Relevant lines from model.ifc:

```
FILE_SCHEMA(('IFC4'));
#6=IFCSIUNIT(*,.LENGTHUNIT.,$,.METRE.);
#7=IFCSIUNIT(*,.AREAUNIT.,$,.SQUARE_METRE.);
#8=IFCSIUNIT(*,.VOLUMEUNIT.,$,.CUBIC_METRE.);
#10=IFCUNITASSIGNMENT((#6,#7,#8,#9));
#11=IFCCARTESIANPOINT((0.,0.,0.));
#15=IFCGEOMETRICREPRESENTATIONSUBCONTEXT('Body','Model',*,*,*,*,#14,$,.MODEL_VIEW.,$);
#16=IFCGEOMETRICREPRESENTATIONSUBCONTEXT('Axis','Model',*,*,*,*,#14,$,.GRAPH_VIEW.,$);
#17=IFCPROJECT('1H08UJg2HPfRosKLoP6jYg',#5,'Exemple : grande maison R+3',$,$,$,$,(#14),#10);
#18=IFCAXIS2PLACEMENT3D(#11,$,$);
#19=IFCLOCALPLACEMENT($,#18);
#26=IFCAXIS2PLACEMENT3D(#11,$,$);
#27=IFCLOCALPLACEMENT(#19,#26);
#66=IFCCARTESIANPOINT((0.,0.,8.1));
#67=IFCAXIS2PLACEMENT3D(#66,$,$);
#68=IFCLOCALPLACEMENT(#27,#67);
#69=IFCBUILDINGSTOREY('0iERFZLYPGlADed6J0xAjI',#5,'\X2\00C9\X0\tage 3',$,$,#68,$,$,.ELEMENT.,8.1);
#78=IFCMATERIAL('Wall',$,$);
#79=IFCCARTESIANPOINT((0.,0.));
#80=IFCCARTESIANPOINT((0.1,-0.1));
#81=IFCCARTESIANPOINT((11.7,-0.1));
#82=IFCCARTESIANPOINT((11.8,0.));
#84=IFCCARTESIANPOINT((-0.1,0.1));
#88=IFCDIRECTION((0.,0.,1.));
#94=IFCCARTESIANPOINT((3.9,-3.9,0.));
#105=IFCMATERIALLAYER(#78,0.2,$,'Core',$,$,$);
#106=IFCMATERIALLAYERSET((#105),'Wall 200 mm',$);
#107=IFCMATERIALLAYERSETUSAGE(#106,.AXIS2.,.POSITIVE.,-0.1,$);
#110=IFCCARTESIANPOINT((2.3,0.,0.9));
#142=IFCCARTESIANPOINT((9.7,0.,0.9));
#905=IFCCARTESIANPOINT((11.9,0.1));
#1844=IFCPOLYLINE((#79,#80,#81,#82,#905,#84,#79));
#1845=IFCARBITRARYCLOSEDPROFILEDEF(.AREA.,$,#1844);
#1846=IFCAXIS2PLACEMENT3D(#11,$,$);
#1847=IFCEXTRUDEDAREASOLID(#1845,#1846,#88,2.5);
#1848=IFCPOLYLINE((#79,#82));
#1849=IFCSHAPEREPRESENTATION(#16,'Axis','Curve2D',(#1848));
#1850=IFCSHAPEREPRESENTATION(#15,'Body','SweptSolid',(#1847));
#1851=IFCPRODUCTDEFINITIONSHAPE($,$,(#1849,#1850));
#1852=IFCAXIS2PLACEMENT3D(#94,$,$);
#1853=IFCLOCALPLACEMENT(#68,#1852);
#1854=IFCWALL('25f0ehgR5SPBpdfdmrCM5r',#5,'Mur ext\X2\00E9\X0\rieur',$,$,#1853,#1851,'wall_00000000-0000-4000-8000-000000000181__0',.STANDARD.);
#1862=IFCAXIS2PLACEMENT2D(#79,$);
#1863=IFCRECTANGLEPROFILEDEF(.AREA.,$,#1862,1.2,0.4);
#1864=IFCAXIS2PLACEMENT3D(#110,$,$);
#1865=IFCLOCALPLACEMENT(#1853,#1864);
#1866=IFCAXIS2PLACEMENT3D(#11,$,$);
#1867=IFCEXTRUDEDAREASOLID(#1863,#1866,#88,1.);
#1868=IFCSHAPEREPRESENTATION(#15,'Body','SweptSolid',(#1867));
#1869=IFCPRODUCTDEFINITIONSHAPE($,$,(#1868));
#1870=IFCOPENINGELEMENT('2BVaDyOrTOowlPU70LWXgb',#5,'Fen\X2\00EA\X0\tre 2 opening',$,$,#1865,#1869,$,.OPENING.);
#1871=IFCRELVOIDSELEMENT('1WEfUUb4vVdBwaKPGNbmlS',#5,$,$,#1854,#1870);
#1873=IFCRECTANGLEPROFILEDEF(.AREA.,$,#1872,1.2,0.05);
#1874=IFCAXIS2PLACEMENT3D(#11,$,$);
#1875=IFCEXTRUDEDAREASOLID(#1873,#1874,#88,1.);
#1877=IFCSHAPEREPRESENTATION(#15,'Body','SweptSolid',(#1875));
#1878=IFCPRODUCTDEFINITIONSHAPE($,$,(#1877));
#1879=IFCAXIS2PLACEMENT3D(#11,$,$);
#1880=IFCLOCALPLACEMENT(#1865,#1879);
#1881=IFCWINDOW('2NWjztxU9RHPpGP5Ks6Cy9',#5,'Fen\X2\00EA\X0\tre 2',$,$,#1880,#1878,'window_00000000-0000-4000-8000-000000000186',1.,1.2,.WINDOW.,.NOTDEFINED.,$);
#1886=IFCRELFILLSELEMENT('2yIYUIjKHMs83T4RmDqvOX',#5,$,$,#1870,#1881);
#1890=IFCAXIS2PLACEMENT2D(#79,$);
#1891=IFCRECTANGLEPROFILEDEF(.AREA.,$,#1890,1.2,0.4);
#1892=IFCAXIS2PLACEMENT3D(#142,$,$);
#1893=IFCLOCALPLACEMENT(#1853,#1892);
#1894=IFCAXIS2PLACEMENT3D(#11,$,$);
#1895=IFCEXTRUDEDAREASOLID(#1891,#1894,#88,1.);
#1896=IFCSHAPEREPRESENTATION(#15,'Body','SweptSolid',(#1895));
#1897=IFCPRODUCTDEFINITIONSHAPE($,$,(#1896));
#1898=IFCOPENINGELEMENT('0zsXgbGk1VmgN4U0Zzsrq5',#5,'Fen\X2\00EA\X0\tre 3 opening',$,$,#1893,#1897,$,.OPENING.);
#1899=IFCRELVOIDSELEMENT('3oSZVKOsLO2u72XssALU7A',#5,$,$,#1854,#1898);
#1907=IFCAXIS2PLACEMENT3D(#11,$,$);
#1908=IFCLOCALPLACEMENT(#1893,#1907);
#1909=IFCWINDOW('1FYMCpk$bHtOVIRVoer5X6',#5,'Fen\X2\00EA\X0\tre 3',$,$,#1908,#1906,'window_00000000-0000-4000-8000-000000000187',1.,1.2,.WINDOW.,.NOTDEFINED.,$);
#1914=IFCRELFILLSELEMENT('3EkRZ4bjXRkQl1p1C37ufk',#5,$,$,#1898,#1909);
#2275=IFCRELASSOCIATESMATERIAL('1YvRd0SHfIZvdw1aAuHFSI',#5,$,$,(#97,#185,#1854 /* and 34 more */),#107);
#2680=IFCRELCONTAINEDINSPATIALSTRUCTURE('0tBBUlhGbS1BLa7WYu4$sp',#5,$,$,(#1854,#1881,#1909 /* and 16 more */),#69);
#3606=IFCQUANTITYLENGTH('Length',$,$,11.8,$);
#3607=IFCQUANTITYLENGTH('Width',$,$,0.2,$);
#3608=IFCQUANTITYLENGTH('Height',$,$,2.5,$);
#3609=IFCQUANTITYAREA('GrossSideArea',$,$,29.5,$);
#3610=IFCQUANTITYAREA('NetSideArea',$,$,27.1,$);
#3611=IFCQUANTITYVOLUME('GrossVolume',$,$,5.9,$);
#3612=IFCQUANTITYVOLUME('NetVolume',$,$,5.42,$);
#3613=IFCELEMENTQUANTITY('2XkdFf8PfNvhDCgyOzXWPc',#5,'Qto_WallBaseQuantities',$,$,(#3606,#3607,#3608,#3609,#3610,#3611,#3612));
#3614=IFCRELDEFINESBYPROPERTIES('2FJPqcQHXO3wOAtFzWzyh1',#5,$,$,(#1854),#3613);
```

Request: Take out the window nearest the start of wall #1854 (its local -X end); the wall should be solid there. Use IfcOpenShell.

```python
import ifcopenshell
import ifcopenshell.api.feature
import ifcopenshell.api.pset
import ifcopenshell.api.root
import ifcopenshell.geom
import ifcopenshell.util.element
import ifcopenshell.util.shape
import ifcopenshell.util.unit

model = ifcopenshell.open("model.ifc")
area_scale = ifcopenshell.util.unit.calculate_unit_scale(model, "AREAUNIT")
volume_scale = ifcopenshell.util.unit.calculate_unit_scale(model, "VOLUMEUNIT")
settings = ifcopenshell.geom.settings()


def volume(element):
    """Net volume in cubic metres, openings subtracted."""
    shape = ifcopenshell.geom.create_shape(settings, element)
    return ifcopenshell.util.shape.get_volume(shape.geometry)


window = model.by_guid("2NWjztxU9RHPpGP5Ks6Cy9")
opening = window.FillsVoids[0].RelatingOpeningElement
wall = opening.VoidsElements[0].RelatingBuildingElement
before = volume(wall)

ifcopenshell.api.root.remove_product(model, product=window)
ifcopenshell.api.feature.remove_feature(model, feature=opening)

after = volume(wall)
thickness = 0.2  # wall thickness in metres

# Update the wall's stored quantities.
qto = model.by_id(ifcopenshell.util.element.get_pset(wall, "Qto_WallBaseQuantities", should_inherit=False)["id"])
ifcopenshell.api.pset.edit_qto(model, qto=qto, properties={
    "NetSideArea": after / thickness / area_scale,
    "NetVolume": after / volume_scale,
})

print(f"wall volume {before:.3f} -> {after:.3f} m3")

model.write("model_edited.ifc")
```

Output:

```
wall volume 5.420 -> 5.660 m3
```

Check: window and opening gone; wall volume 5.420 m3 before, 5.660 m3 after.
